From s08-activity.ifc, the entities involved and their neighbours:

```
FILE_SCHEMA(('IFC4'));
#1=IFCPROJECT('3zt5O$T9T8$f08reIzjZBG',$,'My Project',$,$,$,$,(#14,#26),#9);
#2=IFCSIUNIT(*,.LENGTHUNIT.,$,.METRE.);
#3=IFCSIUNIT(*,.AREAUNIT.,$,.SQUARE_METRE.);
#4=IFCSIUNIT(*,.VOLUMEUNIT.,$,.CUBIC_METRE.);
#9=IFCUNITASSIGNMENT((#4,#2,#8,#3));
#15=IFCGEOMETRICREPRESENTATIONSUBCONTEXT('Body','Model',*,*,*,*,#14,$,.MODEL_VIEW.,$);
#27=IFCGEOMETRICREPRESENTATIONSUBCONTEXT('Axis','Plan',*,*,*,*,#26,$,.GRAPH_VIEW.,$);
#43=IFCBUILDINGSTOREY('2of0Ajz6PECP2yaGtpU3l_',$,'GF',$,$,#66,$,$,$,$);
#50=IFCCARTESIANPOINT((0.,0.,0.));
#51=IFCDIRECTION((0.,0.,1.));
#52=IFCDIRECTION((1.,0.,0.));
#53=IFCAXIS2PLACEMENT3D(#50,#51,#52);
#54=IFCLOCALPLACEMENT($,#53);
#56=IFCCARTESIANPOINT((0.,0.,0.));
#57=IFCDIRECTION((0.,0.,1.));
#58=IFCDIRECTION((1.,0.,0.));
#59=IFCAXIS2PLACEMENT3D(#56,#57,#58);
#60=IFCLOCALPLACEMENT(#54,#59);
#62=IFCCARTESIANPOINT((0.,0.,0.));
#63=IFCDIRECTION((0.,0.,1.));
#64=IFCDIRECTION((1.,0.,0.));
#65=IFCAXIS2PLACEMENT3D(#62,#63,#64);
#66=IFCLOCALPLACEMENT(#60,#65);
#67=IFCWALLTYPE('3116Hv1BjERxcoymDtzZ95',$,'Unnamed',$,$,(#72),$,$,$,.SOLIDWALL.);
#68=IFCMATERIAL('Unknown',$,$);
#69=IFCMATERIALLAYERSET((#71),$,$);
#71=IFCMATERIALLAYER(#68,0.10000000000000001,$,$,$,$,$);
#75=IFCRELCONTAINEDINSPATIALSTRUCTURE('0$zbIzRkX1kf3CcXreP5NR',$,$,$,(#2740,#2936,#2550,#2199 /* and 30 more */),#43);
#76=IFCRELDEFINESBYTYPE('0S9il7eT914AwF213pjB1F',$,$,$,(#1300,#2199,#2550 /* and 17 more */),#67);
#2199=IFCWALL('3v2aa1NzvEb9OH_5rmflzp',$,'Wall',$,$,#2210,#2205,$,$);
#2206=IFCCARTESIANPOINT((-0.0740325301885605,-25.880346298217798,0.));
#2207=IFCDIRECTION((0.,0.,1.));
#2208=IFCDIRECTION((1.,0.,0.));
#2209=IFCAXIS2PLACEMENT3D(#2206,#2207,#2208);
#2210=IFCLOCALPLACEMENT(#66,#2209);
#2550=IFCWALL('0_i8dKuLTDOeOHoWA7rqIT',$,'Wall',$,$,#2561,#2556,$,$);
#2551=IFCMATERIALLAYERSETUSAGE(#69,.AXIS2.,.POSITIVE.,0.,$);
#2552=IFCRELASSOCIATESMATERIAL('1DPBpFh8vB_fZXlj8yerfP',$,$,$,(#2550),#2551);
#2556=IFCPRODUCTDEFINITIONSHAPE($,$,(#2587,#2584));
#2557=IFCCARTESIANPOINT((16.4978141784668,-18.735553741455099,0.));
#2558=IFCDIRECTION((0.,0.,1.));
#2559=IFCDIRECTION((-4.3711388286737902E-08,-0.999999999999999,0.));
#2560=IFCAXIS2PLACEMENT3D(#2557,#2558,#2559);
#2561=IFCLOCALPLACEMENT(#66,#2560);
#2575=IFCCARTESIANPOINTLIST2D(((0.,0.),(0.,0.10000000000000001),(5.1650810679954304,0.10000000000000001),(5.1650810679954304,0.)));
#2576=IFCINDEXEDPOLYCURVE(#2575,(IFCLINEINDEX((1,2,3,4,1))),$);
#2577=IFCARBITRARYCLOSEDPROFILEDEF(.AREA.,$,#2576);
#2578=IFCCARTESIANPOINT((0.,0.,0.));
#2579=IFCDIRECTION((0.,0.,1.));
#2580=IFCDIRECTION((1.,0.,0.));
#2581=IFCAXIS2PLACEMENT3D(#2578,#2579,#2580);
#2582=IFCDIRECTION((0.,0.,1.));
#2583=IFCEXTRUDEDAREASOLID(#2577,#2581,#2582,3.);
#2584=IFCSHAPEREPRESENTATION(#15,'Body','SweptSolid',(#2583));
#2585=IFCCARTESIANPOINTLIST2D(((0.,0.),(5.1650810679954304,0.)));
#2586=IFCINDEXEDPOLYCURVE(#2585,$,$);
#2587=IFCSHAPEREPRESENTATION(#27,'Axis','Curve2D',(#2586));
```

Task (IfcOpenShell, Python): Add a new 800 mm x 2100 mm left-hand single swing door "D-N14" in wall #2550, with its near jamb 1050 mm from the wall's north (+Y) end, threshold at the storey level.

```python
import numpy as np
import ifcopenshell
import ifcopenshell.api.feature
import ifcopenshell.api.geometry
import ifcopenshell.api.root
import ifcopenshell.api.spatial
import ifcopenshell.geom
import ifcopenshell.util.element
import ifcopenshell.util.placement
import ifcopenshell.util.representation
import ifcopenshell.util.shape
import ifcopenshell.util.unit

model = ifcopenshell.open("s08-activity.ifc")
unit_scale = ifcopenshell.util.unit.calculate_unit_scale(model)
settings = ifcopenshell.geom.settings()


def volume(element):
    """Net volume in cubic metres, openings subtracted."""
    shape = ifcopenshell.geom.create_shape(settings, element)
    return ifcopenshell.util.shape.get_volume(shape.geometry)


wall = model.by_guid("0_i8dKuLTDOeOHoWA7rqIT")
storey = ifcopenshell.util.element.get_container(wall, ifc_class="IfcBuildingStorey")
context = ifcopenshell.util.representation.get_context(model, "Model", "Body", "MODEL_VIEW")
before = volume(wall)

width, height, from_end, sill = 0.8, 2.1, 1.05, 0.0  # metres

# The wall runs along its own X axis, and the end named is its -X end.
wall_shape = ifcopenshell.geom.create_shape(settings, wall)
x, y, z = ifcopenshell.util.shape.get_vertices(wall_shape.geometry).T
start = x.min() + from_end
face, thickness = float(y.min()), float(y.max() - y.min())
wall_matrix = ifcopenshell.util.placement.get_local_placement(wall.ObjectPlacement)
level = ifcopenshell.util.placement.get_local_placement(storey.ObjectPlacement)[2, 3]


def in_wall(x, y):
    """Placement at x, y metres in the wall's axes, at sill height."""
    matrix = wall_matrix.copy()
    matrix[:, 3] = wall_matrix @ np.array([x / unit_scale, y / unit_scale, 0.0, 1.0])
    matrix[2, 3] = level + sill / unit_scale
    return matrix


# Opening: a box that overshoots both wall faces by 50 mm.
opening = ifcopenshell.api.root.create_entity(model, ifc_class="IfcOpeningElement", predefined_type="OPENING")
box = ifcopenshell.api.geometry.add_wall_representation(
    model, context=context, length=width, height=height, thickness=thickness + 0.1
)
ifcopenshell.api.geometry.assign_representation(model, product=opening, representation=box)
ifcopenshell.api.geometry.edit_object_placement(model, product=opening, matrix=in_wall(start, face - 0.05), is_si=False)
ifcopenshell.api.feature.add_feature(model, feature=opening, element=wall)

door = ifcopenshell.api.root.create_entity(model, ifc_class="IfcDoor", name="D-N14", predefined_type="DOOR")
door.OverallWidth, door.OverallHeight = width / unit_scale, height / unit_scale
door.OperationType = "SINGLE_SWING_LEFT"
body = ifcopenshell.api.geometry.add_door_representation(
    model,
    context=context,
    overall_width=door.OverallWidth,
    overall_height=door.OverallHeight,
    operation_type="SINGLE_SWING_LEFT",
    lining_properties={"LiningDepth": thickness / unit_scale, "ThresholdDepth": thickness / unit_scale},
)
ifcopenshell.api.geometry.assign_representation(model, product=door, representation=body)
ifcopenshell.api.spatial.assign_container(model, products=[door], relating_structure=storey)
ifcopenshell.api.feature.add_filling(model, opening=opening, element=door)

# The lining spans the wall, so the door starts at the wall face.
ifcopenshell.api.geometry.edit_object_placement(model, product=door, matrix=in_wall(start, face), is_si=False)

after = volume(wall)

print(f"wall volume {before:.3f} -> {after:.3f} m3")

model.write("s08-activity_v2.ifc")
```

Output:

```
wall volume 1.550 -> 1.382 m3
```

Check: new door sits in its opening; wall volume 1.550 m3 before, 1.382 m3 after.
